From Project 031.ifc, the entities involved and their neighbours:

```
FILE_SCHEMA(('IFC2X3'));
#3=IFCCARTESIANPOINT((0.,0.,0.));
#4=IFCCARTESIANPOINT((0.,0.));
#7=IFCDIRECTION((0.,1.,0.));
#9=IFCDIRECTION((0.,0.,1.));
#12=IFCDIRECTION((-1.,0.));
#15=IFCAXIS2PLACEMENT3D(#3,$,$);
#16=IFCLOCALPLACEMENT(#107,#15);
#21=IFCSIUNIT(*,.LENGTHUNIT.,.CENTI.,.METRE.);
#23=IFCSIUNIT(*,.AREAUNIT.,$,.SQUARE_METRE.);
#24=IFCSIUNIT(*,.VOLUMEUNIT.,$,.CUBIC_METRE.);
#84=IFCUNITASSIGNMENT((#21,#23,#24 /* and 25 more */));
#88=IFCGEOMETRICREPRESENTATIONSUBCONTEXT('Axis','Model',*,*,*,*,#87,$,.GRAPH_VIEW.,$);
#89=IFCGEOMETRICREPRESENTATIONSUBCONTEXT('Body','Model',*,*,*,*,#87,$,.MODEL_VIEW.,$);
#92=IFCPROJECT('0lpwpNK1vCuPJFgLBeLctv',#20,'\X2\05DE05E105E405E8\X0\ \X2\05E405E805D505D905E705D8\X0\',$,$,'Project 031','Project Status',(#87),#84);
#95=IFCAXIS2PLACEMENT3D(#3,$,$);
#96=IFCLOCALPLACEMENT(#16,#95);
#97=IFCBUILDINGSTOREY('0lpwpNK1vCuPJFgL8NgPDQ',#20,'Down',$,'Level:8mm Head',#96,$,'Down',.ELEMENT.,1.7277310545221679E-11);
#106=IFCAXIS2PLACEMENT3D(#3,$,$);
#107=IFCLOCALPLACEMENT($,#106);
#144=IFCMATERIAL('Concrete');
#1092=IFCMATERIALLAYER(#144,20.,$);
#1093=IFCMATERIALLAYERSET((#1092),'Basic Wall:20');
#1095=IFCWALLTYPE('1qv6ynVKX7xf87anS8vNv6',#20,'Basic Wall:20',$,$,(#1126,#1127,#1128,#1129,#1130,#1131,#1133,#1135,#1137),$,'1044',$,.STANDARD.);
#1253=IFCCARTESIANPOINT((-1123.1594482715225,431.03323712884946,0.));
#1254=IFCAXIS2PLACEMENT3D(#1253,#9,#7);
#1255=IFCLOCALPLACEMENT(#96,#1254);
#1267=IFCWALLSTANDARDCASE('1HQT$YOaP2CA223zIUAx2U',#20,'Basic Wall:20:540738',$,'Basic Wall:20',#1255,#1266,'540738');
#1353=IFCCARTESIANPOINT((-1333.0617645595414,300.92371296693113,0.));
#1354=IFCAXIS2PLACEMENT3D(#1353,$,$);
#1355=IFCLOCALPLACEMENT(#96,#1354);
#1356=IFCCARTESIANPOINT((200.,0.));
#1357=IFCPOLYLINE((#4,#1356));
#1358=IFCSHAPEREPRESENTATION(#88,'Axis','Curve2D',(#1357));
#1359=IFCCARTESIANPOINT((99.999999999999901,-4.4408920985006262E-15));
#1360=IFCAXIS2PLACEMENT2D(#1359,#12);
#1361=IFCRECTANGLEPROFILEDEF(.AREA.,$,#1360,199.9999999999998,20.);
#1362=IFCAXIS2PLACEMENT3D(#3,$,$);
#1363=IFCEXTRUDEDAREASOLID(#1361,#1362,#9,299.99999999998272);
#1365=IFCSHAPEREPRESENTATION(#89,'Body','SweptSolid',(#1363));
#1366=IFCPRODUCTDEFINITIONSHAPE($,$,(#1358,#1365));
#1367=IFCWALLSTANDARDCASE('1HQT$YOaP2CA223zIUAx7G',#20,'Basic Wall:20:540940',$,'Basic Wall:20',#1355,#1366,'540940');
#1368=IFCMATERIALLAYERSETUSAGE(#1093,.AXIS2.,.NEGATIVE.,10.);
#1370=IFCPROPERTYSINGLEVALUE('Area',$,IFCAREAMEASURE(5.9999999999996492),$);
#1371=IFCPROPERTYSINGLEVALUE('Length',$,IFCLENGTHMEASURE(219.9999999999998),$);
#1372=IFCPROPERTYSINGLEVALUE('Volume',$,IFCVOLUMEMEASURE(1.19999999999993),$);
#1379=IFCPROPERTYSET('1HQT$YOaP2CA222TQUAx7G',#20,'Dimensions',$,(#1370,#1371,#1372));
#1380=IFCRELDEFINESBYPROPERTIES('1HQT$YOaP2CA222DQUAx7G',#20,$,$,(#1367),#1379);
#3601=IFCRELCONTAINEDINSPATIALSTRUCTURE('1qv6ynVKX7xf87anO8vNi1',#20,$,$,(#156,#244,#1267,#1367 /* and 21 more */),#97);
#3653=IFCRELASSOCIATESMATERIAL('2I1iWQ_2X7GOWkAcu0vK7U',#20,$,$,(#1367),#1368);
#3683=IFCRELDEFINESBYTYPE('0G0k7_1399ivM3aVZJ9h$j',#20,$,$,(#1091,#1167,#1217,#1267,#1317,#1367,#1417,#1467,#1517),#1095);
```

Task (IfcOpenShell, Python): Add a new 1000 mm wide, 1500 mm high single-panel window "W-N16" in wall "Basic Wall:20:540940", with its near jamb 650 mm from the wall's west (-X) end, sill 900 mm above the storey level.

```python
import numpy as np
import ifcopenshell
import ifcopenshell.api.feature
import ifcopenshell.api.geometry
import ifcopenshell.api.pset
import ifcopenshell.api.root
import ifcopenshell.api.spatial
import ifcopenshell.api.type
import ifcopenshell.geom
import ifcopenshell.util.element
import ifcopenshell.util.placement
import ifcopenshell.util.representation
import ifcopenshell.util.shape
import ifcopenshell.util.unit

model = ifcopenshell.open("Project 031.ifc")
unit_scale = ifcopenshell.util.unit.calculate_unit_scale(model)
area_scale = ifcopenshell.util.unit.calculate_unit_scale(model, "AREAUNIT")
volume_scale = ifcopenshell.util.unit.calculate_unit_scale(model, "VOLUMEUNIT")
settings = ifcopenshell.geom.settings()


def volume(element):
    """Net volume in cubic metres, openings subtracted."""
    shape = ifcopenshell.geom.create_shape(settings, element)
    return ifcopenshell.util.shape.get_volume(shape.geometry)


wall = model.by_id(1367)
storey = ifcopenshell.util.element.get_container(wall, ifc_class="IfcBuildingStorey")
context = ifcopenshell.util.representation.get_context(model, "Model", "Body", "MODEL_VIEW")
before = volume(wall)

width, height, from_end, sill = 1, 1.5, 0.65, 0.9  # metres

# The wall runs along its own X axis, and the end named is its -X end.
wall_shape = ifcopenshell.geom.create_shape(settings, wall)
x, y, z = ifcopenshell.util.shape.get_vertices(wall_shape.geometry).T
start = x.min() + from_end
face, thickness = float(y.min()), float(y.max() - y.min())
wall_matrix = ifcopenshell.util.placement.get_local_placement(wall.ObjectPlacement)
level = ifcopenshell.util.placement.get_local_placement(storey.ObjectPlacement)[2, 3]


def in_wall(x, y):
    """Placement at x, y metres in the wall's axes, at sill height."""
    matrix = wall_matrix.copy()
    matrix[:, 3] = wall_matrix @ np.array([x / unit_scale, y / unit_scale, 0.0, 1.0])
    matrix[2, 3] = level + sill / unit_scale
    return matrix


# Opening: a box that overshoots both wall faces by 50 mm.
opening = ifcopenshell.api.root.create_entity(model, ifc_class="IfcOpeningElement")
box = ifcopenshell.api.geometry.add_wall_representation(
    model, context=context, length=width, height=height, thickness=thickness + 0.1
)
ifcopenshell.api.geometry.assign_representation(model, product=opening, representation=box)
ifcopenshell.api.geometry.edit_object_placement(model, product=opening, matrix=in_wall(start, face - 0.05), is_si=False)
ifcopenshell.api.feature.add_feature(model, feature=opening, element=wall)

window = ifcopenshell.api.root.create_entity(model, ifc_class="IfcWindow", name="W-N16")
window.OverallWidth, window.OverallHeight = width / unit_scale, height / unit_scale
body = ifcopenshell.api.geometry.add_window_representation(
    model,
    context=context,
    overall_width=window.OverallWidth,
    overall_height=window.OverallHeight,
    partition_type="SINGLE_PANEL",
)
ifcopenshell.api.geometry.assign_representation(model, product=window, representation=body)
ifcopenshell.api.spatial.assign_container(model, products=[window], relating_structure=storey)
fills = ifcopenshell.api.feature.add_filling(model, opening=opening, element=window)
fills.OwnerHistory = window.OwnerHistory  # required in IFC2X3

# IFC2X3 keeps the operation on the window style.
style = ifcopenshell.api.root.create_entity(model, ifc_class="IfcWindowStyle", name="W-N16")
style.OperationType, style.ConstructionType = "SINGLE_PANEL", "NOTDEFINED"
style.ParameterTakesPrecedence = style.Sizeable = False
ifcopenshell.api.type.assign_type(model, related_objects=[window], relating_type=style)

# Centre the window in the wall's thickness.
ifcopenshell.api.geometry.edit_object_placement(model, product=window, matrix=in_wall(start, face), is_si=False)
window_shape = ifcopenshell.geom.create_shape(settings, window)
depth = ifcopenshell.util.shape.get_vertices(window_shape.geometry)[:, 1]
offset = face + thickness / 2 - (depth.min() + depth.max()) / 2
ifcopenshell.api.geometry.edit_object_placement(model, product=window, matrix=in_wall(start, offset), is_si=False)

after = volume(wall)

# Update the wall's stored quantities.
pset = model.by_id(ifcopenshell.util.element.get_pset(wall, "Dimensions", should_inherit=False)["id"])
ifcopenshell.api.pset.edit_pset(model, pset=pset, properties={
    "Area": model.create_entity("IfcAreaMeasure", after / thickness / area_scale),
    "Volume": model.create_entity("IfcVolumeMeasure", after / volume_scale),
})

print(f"wall volume {before:.3f} -> {after:.3f} m3")

model.write("Project 031-out.ifc")
```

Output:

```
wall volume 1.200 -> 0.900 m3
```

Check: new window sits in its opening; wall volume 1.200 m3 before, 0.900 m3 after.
